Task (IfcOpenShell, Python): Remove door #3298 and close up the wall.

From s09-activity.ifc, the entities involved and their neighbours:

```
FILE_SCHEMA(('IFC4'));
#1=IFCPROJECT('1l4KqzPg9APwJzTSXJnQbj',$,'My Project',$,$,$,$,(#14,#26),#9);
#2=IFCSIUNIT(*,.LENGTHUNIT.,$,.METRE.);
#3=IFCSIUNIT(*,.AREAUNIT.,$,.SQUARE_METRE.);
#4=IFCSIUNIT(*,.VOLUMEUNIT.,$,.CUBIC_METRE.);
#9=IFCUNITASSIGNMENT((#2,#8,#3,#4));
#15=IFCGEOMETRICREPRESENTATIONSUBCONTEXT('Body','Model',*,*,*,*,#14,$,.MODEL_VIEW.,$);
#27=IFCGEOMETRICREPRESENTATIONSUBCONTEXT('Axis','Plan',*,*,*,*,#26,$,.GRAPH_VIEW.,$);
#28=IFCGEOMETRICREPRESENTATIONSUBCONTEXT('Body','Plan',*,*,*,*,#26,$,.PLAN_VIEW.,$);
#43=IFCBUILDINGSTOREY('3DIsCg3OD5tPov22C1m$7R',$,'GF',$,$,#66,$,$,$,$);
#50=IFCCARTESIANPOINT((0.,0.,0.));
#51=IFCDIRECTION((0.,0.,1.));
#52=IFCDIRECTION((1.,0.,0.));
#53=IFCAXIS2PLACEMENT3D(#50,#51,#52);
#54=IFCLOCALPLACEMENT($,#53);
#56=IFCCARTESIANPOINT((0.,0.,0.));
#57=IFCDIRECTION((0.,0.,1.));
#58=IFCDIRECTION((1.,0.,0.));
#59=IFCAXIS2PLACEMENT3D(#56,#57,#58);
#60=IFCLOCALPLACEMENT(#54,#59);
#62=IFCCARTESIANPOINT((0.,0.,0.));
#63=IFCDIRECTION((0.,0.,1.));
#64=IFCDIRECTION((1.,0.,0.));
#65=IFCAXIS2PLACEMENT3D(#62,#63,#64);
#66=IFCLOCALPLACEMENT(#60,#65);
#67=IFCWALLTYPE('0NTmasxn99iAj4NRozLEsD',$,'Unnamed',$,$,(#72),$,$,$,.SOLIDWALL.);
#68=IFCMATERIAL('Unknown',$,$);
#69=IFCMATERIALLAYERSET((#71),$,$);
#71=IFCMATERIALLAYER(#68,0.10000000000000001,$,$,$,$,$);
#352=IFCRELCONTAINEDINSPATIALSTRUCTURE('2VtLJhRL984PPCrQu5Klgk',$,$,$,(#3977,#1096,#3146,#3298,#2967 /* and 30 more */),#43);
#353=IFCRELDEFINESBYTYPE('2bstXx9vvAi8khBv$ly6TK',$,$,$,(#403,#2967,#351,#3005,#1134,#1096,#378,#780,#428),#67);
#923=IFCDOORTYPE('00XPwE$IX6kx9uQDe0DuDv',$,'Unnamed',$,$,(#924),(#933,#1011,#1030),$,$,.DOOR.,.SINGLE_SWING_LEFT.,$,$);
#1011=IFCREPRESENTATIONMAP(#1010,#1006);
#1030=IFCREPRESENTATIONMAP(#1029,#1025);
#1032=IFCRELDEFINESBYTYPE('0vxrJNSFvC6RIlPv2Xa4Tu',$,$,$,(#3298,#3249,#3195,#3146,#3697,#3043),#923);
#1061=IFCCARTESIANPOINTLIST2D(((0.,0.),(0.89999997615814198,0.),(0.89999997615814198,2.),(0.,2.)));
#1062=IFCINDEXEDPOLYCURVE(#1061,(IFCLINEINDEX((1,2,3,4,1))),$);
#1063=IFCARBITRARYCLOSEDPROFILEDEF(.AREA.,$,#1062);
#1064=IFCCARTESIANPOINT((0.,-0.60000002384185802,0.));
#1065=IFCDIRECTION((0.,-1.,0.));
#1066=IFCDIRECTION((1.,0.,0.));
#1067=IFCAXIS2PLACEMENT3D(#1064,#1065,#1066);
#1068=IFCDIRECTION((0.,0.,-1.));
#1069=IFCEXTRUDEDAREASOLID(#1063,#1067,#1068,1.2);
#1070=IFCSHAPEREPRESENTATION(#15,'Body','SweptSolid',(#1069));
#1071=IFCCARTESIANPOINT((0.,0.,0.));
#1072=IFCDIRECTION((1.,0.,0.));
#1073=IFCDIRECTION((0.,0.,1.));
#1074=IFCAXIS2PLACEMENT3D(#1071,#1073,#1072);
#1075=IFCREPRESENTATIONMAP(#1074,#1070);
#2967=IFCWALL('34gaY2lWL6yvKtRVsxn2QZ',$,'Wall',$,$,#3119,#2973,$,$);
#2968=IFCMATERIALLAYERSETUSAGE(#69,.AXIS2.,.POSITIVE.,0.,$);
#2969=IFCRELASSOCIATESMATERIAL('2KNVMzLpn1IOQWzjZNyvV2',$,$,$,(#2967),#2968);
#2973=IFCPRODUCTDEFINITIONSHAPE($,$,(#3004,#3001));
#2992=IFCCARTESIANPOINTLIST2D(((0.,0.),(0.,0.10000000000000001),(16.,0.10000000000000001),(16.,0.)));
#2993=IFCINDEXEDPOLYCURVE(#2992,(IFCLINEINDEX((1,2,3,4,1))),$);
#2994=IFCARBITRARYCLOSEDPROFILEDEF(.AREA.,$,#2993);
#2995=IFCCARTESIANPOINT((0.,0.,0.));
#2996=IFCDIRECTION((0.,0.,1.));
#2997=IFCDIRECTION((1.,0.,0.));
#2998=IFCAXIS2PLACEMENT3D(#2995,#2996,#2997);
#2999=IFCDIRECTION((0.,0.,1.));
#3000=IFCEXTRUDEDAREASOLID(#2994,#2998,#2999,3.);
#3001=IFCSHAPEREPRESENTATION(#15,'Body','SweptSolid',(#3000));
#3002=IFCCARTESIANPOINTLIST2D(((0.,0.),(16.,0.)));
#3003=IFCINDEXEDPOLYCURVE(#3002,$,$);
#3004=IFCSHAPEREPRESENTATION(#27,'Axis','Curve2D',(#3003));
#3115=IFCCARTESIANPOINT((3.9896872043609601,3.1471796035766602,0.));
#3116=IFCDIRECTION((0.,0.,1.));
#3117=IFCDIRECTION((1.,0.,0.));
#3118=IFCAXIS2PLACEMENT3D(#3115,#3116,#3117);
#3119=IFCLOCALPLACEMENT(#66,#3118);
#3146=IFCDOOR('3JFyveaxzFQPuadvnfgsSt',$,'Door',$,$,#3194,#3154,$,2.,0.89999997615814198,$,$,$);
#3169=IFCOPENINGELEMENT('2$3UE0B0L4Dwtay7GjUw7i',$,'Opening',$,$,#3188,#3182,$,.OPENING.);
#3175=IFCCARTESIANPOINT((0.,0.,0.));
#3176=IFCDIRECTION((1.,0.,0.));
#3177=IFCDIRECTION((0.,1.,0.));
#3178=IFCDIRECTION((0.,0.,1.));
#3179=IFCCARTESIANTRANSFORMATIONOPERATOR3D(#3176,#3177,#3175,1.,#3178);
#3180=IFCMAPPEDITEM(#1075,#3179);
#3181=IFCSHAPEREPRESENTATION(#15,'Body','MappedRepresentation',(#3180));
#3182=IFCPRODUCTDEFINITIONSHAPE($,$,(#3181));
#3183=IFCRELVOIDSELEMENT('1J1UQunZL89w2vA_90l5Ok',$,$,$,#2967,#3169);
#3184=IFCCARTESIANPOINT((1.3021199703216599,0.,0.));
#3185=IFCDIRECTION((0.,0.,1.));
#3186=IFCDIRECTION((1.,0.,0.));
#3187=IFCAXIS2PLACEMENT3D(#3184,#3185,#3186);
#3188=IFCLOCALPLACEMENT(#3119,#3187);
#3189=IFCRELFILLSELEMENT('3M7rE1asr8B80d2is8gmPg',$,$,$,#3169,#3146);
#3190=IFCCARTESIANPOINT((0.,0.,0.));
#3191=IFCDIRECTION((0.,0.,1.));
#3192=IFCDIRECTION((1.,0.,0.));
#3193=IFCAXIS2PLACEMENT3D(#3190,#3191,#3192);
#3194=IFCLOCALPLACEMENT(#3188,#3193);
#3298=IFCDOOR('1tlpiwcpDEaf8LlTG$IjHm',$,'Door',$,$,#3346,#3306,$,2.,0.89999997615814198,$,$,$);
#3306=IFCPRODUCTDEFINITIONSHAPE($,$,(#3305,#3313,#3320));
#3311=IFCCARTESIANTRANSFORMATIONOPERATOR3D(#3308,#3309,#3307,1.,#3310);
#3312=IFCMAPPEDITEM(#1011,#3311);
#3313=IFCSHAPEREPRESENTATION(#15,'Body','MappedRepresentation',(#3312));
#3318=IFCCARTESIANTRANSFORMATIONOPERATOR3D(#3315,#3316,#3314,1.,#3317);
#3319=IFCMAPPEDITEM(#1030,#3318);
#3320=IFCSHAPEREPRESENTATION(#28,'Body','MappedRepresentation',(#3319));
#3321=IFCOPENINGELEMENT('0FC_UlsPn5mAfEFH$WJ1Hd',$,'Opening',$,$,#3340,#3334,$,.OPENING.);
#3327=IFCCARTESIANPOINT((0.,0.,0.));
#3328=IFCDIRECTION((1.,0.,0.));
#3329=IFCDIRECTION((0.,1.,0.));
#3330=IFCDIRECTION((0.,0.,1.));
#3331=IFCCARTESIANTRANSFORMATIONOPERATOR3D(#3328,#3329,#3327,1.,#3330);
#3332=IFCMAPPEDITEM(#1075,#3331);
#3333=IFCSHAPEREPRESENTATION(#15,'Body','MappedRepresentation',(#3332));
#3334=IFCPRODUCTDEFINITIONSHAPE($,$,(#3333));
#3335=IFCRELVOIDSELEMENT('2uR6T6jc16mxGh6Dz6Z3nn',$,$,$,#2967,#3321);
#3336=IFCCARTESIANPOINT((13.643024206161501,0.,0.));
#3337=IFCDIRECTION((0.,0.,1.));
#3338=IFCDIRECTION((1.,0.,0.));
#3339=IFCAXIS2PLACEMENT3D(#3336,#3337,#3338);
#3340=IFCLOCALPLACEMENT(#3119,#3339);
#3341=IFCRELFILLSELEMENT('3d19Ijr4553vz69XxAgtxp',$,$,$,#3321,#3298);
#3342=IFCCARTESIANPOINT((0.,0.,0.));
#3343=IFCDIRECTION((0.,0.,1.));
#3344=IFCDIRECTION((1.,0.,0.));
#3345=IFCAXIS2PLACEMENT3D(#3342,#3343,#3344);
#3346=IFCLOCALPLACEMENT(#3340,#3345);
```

```python
import ifcopenshell
import ifcopenshell.api.feature
import ifcopenshell.api.root
import ifcopenshell.geom
import ifcopenshell.util.shape

model = ifcopenshell.open("s09-activity.ifc")
settings = ifcopenshell.geom.settings()


def volume(element):
    """Net volume in cubic metres, openings subtracted."""
    shape = ifcopenshell.geom.create_shape(settings, element)
    return ifcopenshell.util.shape.get_volume(shape.geometry)


door = model.by_guid("1tlpiwcpDEaf8LlTG$IjHm")
opening = door.FillsVoids[0].RelatingOpeningElement
wall = opening.VoidsElements[0].RelatingBuildingElement
before = volume(wall)

ifcopenshell.api.root.remove_product(model, product=door)
ifcopenshell.api.feature.remove_feature(model, feature=opening)

after = volume(wall)

print(f"wall volume {before:.3f} -> {after:.3f} m3")

model.write("s09-activity_v2.ifc")
```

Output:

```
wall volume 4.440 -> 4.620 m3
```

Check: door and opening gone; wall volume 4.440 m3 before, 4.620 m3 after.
